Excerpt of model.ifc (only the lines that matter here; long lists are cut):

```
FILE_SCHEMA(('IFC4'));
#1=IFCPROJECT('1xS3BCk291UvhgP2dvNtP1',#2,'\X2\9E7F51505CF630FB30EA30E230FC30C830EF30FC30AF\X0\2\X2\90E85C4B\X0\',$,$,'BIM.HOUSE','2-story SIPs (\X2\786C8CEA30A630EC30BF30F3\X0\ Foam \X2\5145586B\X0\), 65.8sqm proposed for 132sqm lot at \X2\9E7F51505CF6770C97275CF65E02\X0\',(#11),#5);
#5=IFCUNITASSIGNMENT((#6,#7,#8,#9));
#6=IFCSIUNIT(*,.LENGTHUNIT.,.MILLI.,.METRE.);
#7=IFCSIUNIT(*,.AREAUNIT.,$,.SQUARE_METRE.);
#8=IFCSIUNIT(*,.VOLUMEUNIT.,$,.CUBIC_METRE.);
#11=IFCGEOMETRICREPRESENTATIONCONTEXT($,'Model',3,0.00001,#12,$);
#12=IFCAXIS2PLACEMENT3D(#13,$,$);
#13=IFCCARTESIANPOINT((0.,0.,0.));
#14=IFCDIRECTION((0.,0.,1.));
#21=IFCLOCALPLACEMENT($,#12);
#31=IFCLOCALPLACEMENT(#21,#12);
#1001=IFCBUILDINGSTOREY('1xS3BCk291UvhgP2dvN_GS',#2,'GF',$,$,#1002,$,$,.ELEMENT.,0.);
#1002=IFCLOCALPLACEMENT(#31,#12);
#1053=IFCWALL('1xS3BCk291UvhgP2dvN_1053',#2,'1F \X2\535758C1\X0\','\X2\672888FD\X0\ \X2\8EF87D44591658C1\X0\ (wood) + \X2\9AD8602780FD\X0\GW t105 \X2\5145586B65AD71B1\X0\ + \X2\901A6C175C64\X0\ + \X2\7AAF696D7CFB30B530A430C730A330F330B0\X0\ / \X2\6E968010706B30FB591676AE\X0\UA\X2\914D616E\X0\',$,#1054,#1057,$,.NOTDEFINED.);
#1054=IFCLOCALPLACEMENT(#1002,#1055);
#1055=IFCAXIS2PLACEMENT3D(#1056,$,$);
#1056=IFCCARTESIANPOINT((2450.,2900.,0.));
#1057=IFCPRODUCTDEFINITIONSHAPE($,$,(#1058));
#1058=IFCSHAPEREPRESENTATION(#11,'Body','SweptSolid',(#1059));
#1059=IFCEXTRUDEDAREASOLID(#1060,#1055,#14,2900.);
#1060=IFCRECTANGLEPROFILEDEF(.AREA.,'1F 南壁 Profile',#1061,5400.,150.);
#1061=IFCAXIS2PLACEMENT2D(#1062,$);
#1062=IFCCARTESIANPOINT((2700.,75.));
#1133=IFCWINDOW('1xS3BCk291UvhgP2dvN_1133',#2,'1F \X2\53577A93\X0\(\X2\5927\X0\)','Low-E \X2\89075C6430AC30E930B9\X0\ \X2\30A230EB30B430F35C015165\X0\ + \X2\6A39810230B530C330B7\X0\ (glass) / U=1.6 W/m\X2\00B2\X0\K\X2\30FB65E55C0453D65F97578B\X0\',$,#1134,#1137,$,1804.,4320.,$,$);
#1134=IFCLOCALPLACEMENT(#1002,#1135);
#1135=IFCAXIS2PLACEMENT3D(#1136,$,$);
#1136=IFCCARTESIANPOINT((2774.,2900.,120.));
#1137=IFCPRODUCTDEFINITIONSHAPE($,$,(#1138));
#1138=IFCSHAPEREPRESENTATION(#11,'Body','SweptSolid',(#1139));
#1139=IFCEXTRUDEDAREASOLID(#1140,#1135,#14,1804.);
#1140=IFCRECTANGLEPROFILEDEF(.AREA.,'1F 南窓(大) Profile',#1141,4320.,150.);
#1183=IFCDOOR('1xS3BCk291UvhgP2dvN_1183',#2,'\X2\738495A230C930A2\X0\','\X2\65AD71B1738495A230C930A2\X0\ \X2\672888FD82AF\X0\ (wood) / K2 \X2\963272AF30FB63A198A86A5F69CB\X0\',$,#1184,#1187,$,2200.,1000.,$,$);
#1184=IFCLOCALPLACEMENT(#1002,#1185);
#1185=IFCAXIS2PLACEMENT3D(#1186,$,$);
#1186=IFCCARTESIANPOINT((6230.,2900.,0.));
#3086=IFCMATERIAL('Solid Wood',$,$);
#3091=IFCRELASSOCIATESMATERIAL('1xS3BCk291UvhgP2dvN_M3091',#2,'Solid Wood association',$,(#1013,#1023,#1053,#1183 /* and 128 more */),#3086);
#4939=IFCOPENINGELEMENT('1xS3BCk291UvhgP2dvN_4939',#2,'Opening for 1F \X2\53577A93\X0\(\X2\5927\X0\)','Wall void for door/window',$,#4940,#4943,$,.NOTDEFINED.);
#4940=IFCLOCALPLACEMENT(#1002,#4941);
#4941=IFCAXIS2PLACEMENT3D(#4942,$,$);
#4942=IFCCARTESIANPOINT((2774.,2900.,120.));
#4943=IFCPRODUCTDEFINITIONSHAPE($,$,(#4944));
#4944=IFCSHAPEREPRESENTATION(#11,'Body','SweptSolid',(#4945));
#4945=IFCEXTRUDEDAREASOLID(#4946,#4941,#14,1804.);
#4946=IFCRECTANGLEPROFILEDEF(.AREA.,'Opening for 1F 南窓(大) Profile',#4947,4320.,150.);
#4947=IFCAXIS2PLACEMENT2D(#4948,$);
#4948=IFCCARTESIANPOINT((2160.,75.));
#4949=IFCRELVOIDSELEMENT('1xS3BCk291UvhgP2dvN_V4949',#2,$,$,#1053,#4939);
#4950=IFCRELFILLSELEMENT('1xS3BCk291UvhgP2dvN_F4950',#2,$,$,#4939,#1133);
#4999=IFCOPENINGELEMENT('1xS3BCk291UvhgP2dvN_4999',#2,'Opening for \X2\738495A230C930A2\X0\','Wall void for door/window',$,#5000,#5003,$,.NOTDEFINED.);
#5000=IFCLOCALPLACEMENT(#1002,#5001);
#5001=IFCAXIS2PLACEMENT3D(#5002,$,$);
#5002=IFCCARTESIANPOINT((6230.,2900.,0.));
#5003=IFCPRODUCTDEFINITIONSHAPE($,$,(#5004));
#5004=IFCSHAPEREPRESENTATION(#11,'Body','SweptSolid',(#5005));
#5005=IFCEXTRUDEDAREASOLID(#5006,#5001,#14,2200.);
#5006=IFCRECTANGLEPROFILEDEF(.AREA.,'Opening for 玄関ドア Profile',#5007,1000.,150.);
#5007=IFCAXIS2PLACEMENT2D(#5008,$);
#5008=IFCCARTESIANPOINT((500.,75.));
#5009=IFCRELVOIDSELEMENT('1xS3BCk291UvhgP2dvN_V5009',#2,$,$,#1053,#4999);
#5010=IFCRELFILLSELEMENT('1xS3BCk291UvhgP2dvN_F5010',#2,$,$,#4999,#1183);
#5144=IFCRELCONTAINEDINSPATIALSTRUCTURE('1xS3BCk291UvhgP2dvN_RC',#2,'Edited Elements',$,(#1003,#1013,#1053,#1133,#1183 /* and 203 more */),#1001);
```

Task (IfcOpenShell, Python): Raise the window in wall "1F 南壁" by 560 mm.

```python
import numpy as np
import ifcopenshell
import ifcopenshell.api.geometry
import ifcopenshell.util.placement
import ifcopenshell.util.unit

model = ifcopenshell.open("model.ifc")
unit_scale = ifcopenshell.util.unit.calculate_unit_scale(model)

window = model.by_guid("1xS3BCk291UvhgP2dvN_1133")
opening = window.FillsVoids[0].RelatingOpeningElement
dz = 0.56 / unit_scale

shift = np.array([0.0, 0.0, dz])
# The window is not placed relative to its opening, so move both.
for product in (opening, window):
    matrix = ifcopenshell.util.placement.get_local_placement(product.ObjectPlacement)
    matrix[:3, 3] += shift
    ifcopenshell.api.geometry.edit_object_placement(model, product=product, matrix=matrix, is_si=False)

print(f"moved by {dz * unit_scale:+.3f} m")

model.write("model_rev.ifc")
```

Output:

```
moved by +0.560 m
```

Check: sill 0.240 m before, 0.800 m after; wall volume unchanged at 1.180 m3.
